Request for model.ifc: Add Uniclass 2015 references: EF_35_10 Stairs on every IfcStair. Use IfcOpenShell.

First a look at what the model holds.

```python
import ifcopenshell

model = ifcopenshell.open("model.ifc")
print(model.schema)
print("classifications:", [c.Name for c in model.by_type("IfcClassification")])
for ifc_class in ("IfcDoor", "IfcRoof", "IfcStair", "IfcWall", "IfcWindow"):
    print(ifc_class, len(model.by_type(ifc_class)))
```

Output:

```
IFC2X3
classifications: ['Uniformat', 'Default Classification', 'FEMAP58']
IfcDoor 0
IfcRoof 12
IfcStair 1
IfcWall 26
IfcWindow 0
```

```python
import ifcopenshell
import ifcopenshell.api.classification

model = ifcopenshell.open("model.ifc")

# IFC2X3 requires Source and Edition and has no link from the project to the system.
system = model.create_entity("IfcClassification", Source="NBS", Edition="2015", Name="Uniclass 2015")

codes = {
    "IfcStair": ("EF_35_10", "Stairs"),
}
for ifc_class, (code, name) in codes.items():
    products = model.by_type(ifc_class)
    ifcopenshell.api.classification.add_reference(
        model, products=products, classification=system, identification=code, name=name
    )
    print(code, len(products))

model.write("model-out.ifc")
```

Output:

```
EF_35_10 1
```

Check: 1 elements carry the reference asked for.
